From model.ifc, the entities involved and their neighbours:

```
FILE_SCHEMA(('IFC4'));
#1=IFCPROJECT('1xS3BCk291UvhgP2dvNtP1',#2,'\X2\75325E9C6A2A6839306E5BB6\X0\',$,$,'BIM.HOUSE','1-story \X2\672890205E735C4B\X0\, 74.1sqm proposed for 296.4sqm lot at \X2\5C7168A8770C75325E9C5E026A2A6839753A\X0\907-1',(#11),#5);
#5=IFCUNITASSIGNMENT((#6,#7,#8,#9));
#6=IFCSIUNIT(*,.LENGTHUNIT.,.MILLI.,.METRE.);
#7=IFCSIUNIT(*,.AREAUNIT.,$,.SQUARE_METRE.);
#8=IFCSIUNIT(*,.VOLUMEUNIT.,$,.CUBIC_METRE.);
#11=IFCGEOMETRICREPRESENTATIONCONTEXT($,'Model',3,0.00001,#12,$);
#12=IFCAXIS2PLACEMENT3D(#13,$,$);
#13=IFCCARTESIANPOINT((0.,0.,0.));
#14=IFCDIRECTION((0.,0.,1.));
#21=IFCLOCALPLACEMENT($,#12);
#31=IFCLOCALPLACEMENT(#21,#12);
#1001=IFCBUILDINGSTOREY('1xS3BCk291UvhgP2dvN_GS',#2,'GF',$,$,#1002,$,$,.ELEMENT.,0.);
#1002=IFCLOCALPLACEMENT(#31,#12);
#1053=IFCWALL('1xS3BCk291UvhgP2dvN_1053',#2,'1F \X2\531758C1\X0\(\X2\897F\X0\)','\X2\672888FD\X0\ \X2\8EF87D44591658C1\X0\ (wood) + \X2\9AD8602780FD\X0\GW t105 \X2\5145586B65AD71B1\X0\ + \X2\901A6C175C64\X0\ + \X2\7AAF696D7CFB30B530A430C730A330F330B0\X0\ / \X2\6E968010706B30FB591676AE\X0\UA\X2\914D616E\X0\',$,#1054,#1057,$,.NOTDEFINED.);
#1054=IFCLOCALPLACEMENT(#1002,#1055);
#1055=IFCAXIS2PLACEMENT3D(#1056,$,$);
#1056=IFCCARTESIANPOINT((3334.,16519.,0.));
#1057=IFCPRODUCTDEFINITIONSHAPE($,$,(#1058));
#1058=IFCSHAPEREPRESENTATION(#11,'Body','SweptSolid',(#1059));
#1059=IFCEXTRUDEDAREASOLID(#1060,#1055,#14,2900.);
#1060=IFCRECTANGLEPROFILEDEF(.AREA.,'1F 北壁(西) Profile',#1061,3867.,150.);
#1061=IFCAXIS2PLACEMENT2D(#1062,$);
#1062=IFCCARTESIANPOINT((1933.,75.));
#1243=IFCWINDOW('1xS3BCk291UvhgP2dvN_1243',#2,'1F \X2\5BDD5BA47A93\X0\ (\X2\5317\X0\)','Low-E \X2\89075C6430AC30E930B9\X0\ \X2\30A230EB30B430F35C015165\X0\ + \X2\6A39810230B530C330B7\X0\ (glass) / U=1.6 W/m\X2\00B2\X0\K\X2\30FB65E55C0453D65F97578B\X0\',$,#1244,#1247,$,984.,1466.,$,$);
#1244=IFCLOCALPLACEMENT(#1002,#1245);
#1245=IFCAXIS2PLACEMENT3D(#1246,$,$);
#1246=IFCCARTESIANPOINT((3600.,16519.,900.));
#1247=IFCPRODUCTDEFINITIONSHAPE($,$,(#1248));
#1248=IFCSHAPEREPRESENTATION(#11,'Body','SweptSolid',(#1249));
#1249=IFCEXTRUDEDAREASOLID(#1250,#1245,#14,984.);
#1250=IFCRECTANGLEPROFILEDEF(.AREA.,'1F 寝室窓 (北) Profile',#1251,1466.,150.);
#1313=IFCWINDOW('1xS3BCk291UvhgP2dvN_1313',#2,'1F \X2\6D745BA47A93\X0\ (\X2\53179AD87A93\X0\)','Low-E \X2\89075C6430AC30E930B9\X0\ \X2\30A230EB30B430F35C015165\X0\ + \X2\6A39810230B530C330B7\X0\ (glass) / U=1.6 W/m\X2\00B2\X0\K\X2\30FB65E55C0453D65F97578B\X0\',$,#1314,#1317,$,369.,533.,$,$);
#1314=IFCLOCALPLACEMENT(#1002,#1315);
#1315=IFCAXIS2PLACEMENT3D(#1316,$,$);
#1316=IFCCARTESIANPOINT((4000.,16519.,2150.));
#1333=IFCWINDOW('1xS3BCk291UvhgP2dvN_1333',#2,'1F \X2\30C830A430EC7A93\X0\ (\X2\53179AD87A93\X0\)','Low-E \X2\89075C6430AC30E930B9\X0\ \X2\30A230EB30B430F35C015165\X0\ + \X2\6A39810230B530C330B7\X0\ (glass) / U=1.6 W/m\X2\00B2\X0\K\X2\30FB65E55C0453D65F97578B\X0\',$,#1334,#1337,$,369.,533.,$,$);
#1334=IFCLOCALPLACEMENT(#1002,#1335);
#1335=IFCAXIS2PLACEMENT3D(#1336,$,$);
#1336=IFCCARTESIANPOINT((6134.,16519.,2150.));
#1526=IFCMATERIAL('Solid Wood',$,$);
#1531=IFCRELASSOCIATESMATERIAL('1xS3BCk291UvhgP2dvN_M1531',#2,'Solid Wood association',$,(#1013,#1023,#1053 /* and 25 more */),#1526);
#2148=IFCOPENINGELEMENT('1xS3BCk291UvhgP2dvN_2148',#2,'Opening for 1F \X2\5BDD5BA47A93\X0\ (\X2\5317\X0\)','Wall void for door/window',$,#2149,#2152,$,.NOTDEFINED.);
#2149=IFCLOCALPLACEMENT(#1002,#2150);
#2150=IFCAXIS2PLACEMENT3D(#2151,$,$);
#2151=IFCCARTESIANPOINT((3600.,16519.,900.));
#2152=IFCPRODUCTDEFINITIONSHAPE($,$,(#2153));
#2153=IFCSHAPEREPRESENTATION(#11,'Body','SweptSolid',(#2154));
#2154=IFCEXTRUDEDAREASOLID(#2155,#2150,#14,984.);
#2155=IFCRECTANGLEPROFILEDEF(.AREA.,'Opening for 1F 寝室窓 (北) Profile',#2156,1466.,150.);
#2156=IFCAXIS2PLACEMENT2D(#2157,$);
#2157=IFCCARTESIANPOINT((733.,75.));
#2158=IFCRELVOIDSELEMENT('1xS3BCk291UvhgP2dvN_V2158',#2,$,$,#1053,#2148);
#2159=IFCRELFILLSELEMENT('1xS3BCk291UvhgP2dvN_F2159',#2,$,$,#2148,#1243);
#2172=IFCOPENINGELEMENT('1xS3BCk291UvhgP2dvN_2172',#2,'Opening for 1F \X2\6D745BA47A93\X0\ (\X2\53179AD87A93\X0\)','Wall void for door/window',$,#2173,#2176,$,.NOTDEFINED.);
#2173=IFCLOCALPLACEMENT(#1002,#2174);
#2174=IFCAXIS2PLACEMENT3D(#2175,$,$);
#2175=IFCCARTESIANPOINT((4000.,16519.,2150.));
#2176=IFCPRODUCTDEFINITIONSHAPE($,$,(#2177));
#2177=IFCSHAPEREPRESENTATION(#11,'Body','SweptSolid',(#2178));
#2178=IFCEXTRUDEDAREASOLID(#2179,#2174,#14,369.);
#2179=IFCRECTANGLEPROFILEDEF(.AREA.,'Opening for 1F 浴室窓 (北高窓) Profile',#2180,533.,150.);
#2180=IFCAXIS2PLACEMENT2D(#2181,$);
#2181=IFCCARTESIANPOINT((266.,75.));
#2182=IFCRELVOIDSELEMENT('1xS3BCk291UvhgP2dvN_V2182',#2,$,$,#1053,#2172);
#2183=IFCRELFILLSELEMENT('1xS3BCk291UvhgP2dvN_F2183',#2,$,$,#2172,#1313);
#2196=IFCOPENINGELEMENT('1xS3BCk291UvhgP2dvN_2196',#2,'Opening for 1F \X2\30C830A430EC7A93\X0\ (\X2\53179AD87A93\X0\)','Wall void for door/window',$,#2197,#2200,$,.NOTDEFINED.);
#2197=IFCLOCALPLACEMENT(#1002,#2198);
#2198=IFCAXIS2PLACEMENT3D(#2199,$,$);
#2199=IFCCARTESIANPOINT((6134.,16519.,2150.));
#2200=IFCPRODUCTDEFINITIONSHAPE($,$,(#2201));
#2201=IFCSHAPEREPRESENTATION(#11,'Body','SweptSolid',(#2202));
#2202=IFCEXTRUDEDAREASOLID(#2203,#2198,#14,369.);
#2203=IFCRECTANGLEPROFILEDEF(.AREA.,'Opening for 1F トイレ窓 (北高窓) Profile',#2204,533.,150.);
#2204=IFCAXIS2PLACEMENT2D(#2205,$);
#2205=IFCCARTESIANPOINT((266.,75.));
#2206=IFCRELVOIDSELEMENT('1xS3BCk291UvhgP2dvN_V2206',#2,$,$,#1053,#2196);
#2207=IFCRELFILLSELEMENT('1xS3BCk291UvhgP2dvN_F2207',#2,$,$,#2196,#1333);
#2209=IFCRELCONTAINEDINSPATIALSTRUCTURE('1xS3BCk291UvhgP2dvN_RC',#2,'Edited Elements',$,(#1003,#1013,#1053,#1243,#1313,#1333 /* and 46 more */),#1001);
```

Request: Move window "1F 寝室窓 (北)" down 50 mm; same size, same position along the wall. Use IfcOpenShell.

```python
import numpy as np
import ifcopenshell
import ifcopenshell.api.geometry
import ifcopenshell.util.placement
import ifcopenshell.util.unit

model = ifcopenshell.open("model.ifc")
unit_scale = ifcopenshell.util.unit.calculate_unit_scale(model)

window = model.by_guid("1xS3BCk291UvhgP2dvN_1243")
opening = window.FillsVoids[0].RelatingOpeningElement
dz = -50.0

shift = np.array([0.0, 0.0, dz])
# The window is not placed relative to its opening, so move both.
for product in (opening, window):
    matrix = ifcopenshell.util.placement.get_local_placement(product.ObjectPlacement)
    matrix[:3, 3] += shift
    ifcopenshell.api.geometry.edit_object_placement(model, product=product, matrix=matrix, is_si=False)

print(f"moved by {dz * unit_scale:+.3f} m")

model.write("model_v2.ifc")
```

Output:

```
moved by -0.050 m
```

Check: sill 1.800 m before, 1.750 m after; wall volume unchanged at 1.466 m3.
